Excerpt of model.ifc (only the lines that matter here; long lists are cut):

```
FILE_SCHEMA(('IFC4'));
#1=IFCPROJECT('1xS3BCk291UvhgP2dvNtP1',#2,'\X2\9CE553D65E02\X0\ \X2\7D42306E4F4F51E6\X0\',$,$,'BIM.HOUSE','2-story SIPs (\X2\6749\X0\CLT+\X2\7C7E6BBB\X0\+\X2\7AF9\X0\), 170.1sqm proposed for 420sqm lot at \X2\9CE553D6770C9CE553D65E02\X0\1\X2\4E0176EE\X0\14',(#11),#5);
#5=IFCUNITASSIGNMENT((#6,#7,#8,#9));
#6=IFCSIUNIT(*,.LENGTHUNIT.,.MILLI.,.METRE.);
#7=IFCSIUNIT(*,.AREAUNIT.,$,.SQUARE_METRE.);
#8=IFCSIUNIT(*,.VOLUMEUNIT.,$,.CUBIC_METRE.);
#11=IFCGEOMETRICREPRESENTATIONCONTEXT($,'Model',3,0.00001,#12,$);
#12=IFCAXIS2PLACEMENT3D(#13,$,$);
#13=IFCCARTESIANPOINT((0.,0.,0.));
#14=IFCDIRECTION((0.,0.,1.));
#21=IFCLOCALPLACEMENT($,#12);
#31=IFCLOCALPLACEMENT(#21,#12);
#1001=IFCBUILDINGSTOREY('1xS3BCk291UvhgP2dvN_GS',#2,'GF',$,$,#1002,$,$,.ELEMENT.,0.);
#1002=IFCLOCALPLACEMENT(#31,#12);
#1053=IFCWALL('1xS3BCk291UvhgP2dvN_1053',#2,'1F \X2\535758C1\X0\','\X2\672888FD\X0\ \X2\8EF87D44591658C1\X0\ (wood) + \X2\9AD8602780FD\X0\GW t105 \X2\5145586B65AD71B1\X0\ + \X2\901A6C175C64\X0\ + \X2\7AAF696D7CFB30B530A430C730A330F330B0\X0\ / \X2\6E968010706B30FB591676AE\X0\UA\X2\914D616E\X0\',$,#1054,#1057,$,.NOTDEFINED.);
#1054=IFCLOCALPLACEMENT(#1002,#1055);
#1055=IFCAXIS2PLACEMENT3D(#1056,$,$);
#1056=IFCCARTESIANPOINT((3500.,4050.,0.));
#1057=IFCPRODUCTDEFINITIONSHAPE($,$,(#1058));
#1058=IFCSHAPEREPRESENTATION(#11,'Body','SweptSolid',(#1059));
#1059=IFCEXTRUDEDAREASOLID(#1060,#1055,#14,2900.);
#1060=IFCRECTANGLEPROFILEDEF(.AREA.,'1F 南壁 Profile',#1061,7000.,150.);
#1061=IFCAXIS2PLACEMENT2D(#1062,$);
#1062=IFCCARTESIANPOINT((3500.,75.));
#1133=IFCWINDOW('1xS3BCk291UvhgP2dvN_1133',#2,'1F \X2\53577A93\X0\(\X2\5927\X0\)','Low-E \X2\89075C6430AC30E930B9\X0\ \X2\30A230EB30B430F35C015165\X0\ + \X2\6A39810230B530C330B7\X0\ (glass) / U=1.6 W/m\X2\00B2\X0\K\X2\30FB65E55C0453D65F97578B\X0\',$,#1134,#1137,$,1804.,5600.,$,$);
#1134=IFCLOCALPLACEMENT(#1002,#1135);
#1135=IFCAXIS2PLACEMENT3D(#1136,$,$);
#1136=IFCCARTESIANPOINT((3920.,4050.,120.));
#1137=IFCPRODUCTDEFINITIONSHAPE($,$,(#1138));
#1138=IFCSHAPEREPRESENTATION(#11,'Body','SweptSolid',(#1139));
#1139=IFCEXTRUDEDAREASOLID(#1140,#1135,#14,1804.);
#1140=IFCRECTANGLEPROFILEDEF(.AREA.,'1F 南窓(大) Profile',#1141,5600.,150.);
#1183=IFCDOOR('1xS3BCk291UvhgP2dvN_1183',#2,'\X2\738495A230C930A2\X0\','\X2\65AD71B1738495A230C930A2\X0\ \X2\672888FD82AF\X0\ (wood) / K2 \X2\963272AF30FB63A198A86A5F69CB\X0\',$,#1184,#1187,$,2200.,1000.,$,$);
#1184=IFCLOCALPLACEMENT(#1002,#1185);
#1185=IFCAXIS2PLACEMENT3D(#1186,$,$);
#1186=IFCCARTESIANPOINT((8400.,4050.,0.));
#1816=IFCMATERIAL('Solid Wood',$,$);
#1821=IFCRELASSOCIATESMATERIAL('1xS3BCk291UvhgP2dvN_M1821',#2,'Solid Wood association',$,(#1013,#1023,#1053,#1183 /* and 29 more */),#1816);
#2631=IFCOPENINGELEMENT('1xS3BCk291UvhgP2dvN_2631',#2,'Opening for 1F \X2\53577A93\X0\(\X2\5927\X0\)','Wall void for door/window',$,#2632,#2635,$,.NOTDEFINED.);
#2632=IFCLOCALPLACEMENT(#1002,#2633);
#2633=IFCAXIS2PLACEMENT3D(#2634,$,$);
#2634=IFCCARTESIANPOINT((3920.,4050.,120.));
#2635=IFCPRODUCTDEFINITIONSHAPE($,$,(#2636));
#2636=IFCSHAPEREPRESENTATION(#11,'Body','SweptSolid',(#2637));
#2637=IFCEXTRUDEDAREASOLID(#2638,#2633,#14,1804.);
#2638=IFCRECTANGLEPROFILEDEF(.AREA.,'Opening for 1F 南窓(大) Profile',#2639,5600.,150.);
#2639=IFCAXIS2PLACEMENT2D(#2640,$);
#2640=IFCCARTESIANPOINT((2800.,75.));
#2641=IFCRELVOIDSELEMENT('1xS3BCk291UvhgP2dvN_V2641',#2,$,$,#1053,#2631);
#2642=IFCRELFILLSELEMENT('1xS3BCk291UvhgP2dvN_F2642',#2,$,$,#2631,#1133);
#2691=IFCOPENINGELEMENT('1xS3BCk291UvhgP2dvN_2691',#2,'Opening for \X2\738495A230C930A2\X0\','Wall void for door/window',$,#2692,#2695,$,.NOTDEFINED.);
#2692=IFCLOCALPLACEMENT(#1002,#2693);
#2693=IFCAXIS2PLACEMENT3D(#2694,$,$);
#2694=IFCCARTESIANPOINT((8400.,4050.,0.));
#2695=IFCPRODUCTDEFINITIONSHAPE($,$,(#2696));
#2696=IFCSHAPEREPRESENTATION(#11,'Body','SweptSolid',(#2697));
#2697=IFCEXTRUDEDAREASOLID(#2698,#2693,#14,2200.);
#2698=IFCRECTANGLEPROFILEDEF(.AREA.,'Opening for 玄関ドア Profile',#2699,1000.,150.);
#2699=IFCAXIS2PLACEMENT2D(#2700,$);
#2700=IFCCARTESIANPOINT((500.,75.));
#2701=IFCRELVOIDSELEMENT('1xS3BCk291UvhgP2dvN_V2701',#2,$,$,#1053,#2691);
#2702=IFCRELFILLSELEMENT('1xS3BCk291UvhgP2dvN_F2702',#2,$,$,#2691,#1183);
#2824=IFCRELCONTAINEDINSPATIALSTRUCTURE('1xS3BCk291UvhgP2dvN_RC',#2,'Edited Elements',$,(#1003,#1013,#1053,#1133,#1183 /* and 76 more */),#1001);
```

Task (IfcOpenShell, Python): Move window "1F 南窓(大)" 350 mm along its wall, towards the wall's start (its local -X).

```python
import ifcopenshell
import ifcopenshell.api.geometry
import ifcopenshell.util.placement
import ifcopenshell.util.unit

model = ifcopenshell.open("model.ifc")
unit_scale = ifcopenshell.util.unit.calculate_unit_scale(model)

window = model.by_guid("1xS3BCk291UvhgP2dvN_1133")
opening = window.FillsVoids[0].RelatingOpeningElement
wall = opening.VoidsElements[0].RelatingBuildingElement

wall_matrix = ifcopenshell.util.placement.get_local_placement(wall.ObjectPlacement)
shift = wall_matrix[:3, 0] * -0.35 / unit_scale
before = ifcopenshell.util.placement.get_local_placement(window.ObjectPlacement)[:3, 3].copy()

# The window is not placed relative to its opening, so move both.
for product in (opening, window):
    matrix = ifcopenshell.util.placement.get_local_placement(product.ObjectPlacement)
    matrix[:3, 3] += shift
    ifcopenshell.api.geometry.edit_object_placement(model, product=product, matrix=matrix, is_si=False)

after = ifcopenshell.util.placement.get_local_placement(window.ObjectPlacement)[:3, 3]
print("window moved by", (after - before).round(3) + 0.0)

model.write("model_v2.ifc")
```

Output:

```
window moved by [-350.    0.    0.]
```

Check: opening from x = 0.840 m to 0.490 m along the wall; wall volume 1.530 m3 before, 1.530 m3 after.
